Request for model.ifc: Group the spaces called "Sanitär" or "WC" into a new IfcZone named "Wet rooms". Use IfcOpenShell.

First a look at what the model holds.

```python
import ifcopenshell

model = ifcopenshell.open("model.ifc")
print(model.schema)
seen = {}
for space in model.by_type("IfcSpace"):
    seen[space.LongName] = seen.get(space.LongName, 0) + 1
for name, count in sorted(seen.items(), key=str):
    print(count, "x", name)
print("zones:", [z.Name for z in model.by_type("IfcZone")][:20])
```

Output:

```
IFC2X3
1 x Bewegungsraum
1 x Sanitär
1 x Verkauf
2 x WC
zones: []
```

```python
import ifcopenshell
import ifcopenshell.api.group
import ifcopenshell.api.root

model = ifcopenshell.open("model.ifc")

names = {"Sanitär", "WC"}
spaces = [s for s in model.by_type("IfcSpace") if s.LongName in names]

zone = ifcopenshell.api.root.create_entity(model, ifc_class="IfcZone", name="Wet rooms")
ifcopenshell.api.group.assign_group(model, products=spaces, group=zone)
print(len(spaces), "spaces in", zone.Name)

model.write("model_rev.ifc")
```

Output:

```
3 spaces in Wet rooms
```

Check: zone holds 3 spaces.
